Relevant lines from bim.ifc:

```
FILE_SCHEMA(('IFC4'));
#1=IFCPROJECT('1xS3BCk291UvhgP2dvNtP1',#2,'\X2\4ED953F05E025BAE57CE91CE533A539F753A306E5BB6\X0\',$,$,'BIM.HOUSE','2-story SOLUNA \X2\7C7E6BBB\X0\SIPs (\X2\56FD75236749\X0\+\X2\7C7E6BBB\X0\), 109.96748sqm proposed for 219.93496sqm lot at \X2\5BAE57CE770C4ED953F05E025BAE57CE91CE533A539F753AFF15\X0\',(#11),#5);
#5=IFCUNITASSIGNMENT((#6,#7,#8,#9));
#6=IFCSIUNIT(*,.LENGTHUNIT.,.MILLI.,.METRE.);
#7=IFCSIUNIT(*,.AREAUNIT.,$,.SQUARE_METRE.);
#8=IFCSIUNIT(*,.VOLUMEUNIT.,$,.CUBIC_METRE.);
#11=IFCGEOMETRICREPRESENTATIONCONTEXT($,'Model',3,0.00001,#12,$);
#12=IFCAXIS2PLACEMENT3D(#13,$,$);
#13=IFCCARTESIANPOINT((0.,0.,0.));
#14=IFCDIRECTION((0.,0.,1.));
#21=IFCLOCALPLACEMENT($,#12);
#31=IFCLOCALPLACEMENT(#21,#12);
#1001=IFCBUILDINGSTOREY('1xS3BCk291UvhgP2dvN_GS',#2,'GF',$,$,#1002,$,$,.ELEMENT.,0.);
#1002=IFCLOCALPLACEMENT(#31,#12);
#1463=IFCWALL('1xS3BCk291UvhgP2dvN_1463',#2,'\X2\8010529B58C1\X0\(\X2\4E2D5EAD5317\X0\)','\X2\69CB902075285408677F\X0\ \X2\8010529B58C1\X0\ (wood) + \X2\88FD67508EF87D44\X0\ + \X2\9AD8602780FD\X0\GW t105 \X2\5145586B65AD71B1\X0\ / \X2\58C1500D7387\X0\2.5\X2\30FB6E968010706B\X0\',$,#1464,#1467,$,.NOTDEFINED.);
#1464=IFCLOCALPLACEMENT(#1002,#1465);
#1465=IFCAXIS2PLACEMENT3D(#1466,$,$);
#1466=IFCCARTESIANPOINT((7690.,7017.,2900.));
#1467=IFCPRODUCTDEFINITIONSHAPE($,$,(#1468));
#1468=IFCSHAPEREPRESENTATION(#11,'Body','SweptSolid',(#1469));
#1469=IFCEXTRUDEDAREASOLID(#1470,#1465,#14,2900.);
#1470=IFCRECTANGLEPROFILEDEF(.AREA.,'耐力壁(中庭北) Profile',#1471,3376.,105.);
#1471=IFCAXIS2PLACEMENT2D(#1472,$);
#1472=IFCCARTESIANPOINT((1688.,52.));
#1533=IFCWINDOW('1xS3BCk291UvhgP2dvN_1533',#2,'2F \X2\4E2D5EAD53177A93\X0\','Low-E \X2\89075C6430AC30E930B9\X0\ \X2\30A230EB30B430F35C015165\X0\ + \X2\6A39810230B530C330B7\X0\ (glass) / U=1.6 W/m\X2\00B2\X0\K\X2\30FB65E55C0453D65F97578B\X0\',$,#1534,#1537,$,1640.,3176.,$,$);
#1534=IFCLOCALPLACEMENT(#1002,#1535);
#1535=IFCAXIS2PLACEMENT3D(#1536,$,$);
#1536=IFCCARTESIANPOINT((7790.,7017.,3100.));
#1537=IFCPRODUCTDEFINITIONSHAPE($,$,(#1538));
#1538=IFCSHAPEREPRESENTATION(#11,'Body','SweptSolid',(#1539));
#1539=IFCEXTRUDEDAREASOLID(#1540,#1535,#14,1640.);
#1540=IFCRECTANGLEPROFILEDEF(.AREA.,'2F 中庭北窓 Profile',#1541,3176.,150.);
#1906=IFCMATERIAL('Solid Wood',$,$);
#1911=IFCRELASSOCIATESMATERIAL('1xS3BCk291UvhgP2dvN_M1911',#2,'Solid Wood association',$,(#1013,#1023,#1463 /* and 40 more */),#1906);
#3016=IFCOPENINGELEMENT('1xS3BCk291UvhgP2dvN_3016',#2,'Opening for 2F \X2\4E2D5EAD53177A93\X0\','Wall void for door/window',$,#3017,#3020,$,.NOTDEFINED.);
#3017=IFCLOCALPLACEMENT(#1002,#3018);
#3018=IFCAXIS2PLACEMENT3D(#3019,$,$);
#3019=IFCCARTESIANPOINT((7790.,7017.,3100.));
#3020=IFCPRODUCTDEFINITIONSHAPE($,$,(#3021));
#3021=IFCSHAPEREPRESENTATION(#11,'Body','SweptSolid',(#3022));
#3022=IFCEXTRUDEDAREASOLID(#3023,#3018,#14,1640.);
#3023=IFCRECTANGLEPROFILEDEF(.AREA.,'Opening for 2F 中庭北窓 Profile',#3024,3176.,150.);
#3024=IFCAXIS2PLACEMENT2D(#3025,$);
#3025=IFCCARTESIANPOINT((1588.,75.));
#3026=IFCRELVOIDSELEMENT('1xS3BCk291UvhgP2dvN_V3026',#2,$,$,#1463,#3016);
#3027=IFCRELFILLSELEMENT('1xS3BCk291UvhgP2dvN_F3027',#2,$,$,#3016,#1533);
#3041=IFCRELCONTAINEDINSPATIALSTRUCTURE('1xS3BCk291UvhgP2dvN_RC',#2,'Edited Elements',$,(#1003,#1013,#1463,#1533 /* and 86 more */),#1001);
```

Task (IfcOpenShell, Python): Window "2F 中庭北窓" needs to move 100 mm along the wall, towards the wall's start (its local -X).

```python
import ifcopenshell
import ifcopenshell.api.geometry
import ifcopenshell.util.placement

model = ifcopenshell.open("bim.ifc")

window = model.by_guid("1xS3BCk291UvhgP2dvN_1533")
opening = window.FillsVoids[0].RelatingOpeningElement
wall = opening.VoidsElements[0].RelatingBuildingElement

wall_matrix = ifcopenshell.util.placement.get_local_placement(wall.ObjectPlacement)
shift = wall_matrix[:3, 0] * -100.0
before = ifcopenshell.util.placement.get_local_placement(window.ObjectPlacement)[:3, 3].copy()

# The window is not placed relative to its opening, so move both.
for product in (opening, window):
    matrix = ifcopenshell.util.placement.get_local_placement(product.ObjectPlacement)
    matrix[:3, 3] += shift
    ifcopenshell.api.geometry.edit_object_placement(model, product=product, matrix=matrix, is_si=False)

after = ifcopenshell.util.placement.get_local_placement(window.ObjectPlacement)[:3, 3]
print("window moved by", (after - before).round(3) + 0.0)

model.write("bim_edited.ifc")
```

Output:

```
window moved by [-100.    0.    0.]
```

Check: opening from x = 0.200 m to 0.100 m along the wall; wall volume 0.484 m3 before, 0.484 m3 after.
